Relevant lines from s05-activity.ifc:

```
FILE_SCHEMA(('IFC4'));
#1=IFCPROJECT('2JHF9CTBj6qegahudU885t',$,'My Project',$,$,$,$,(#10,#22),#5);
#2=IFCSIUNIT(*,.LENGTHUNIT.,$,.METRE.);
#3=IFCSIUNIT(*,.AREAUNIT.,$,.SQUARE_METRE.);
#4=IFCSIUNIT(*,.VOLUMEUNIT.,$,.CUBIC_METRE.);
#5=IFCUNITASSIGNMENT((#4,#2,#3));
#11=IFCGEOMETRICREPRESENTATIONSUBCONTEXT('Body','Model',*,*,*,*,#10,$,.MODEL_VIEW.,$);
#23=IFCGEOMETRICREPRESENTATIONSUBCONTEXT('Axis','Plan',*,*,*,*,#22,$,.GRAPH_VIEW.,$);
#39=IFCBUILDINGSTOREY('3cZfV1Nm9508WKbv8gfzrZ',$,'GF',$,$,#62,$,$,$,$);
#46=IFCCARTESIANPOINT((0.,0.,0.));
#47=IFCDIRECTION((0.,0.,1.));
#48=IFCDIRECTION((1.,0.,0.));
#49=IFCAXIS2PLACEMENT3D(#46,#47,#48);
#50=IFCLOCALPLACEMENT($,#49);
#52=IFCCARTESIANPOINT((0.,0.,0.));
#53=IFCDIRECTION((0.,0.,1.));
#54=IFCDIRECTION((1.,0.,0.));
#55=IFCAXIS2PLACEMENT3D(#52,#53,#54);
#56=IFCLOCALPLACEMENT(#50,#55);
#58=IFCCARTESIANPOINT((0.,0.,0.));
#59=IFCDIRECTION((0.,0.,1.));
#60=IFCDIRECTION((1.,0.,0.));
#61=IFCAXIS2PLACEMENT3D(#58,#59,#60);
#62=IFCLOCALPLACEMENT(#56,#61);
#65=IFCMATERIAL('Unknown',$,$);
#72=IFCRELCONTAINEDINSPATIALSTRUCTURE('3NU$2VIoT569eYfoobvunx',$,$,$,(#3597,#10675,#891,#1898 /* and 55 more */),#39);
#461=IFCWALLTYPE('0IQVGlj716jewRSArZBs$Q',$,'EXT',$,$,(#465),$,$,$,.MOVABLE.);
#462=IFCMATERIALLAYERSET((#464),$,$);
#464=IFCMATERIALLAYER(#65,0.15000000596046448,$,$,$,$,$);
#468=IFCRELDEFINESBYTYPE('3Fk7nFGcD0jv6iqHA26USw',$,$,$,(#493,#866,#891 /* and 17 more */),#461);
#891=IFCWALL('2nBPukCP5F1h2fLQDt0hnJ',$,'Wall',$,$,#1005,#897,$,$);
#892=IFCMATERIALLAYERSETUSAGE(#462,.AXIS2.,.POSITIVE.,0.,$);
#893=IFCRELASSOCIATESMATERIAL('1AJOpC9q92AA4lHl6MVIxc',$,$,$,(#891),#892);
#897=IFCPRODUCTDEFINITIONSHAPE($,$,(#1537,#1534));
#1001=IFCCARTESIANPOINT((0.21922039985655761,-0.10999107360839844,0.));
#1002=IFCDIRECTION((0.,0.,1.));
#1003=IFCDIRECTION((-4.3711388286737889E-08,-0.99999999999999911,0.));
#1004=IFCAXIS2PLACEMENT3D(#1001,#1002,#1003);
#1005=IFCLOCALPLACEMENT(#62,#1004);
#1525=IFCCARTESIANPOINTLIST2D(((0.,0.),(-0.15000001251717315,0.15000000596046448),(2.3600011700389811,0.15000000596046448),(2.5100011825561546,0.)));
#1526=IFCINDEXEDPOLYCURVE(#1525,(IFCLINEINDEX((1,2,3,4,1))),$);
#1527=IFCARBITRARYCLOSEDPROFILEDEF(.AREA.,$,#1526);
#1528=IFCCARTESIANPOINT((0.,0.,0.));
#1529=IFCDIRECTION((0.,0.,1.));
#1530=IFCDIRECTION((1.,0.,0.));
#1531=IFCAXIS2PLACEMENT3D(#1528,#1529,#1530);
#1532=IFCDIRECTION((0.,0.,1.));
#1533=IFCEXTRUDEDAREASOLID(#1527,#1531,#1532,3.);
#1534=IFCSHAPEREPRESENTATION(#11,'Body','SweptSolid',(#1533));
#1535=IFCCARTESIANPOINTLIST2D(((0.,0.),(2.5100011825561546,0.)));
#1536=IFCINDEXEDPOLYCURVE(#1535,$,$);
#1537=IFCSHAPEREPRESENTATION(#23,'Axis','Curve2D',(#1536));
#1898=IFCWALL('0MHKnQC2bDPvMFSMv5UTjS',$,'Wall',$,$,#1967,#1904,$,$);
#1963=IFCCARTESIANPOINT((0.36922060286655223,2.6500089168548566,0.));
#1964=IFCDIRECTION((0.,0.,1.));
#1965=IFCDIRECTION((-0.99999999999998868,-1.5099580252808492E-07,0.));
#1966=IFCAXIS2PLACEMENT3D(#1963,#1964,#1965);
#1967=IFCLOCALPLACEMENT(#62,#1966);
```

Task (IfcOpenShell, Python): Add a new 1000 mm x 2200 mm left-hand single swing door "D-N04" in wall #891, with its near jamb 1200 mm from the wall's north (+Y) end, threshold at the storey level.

```python
import numpy as np
import ifcopenshell
import ifcopenshell.api.feature
import ifcopenshell.api.geometry
import ifcopenshell.api.root
import ifcopenshell.api.spatial
import ifcopenshell.geom
import ifcopenshell.util.element
import ifcopenshell.util.placement
import ifcopenshell.util.representation
import ifcopenshell.util.shape
import ifcopenshell.util.unit

model = ifcopenshell.open("s05-activity.ifc")
unit_scale = ifcopenshell.util.unit.calculate_unit_scale(model)
settings = ifcopenshell.geom.settings()


def volume(element):
    """Net volume in cubic metres, openings subtracted."""
    shape = ifcopenshell.geom.create_shape(settings, element)
    return ifcopenshell.util.shape.get_volume(shape.geometry)


wall = model.by_guid("2nBPukCP5F1h2fLQDt0hnJ")
storey = ifcopenshell.util.element.get_container(wall, ifc_class="IfcBuildingStorey")
context = ifcopenshell.util.representation.get_context(model, "Model", "Body", "MODEL_VIEW")
before = volume(wall)

width, height, from_end, sill = 1, 2.2, 1.2, 0.0  # metres

# The wall runs along its own X axis, and the end named is its -X end.
wall_shape = ifcopenshell.geom.create_shape(settings, wall)
x, y, z = ifcopenshell.util.shape.get_vertices(wall_shape.geometry).T
start = x.min() + from_end
face, thickness = float(y.min()), float(y.max() - y.min())
wall_matrix = ifcopenshell.util.placement.get_local_placement(wall.ObjectPlacement)
level = ifcopenshell.util.placement.get_local_placement(storey.ObjectPlacement)[2, 3]


def in_wall(x, y):
    """Placement at x, y metres in the wall's axes, at sill height."""
    matrix = wall_matrix.copy()
    matrix[:, 3] = wall_matrix @ np.array([x / unit_scale, y / unit_scale, 0.0, 1.0])
    matrix[2, 3] = level + sill / unit_scale
    return matrix


# Opening: a box that overshoots both wall faces by 50 mm.
opening = ifcopenshell.api.root.create_entity(model, ifc_class="IfcOpeningElement", predefined_type="OPENING")
box = ifcopenshell.api.geometry.add_wall_representation(
    model, context=context, length=width, height=height, thickness=thickness + 0.1
)
ifcopenshell.api.geometry.assign_representation(model, product=opening, representation=box)
ifcopenshell.api.geometry.edit_object_placement(model, product=opening, matrix=in_wall(start, face - 0.05), is_si=False)
ifcopenshell.api.feature.add_feature(model, feature=opening, element=wall)

door = ifcopenshell.api.root.create_entity(model, ifc_class="IfcDoor", name="D-N04", predefined_type="DOOR")
door.OverallWidth, door.OverallHeight = width / unit_scale, height / unit_scale
door.OperationType = "SINGLE_SWING_LEFT"
body = ifcopenshell.api.geometry.add_door_representation(
    model,
    context=context,
    overall_width=door.OverallWidth,
    overall_height=door.OverallHeight,
    operation_type="SINGLE_SWING_LEFT",
    lining_properties={"LiningDepth": thickness / unit_scale, "ThresholdDepth": thickness / unit_scale},
)
ifcopenshell.api.geometry.assign_representation(model, product=door, representation=body)
ifcopenshell.api.spatial.assign_container(model, products=[door], relating_structure=storey)
ifcopenshell.api.feature.add_filling(model, opening=opening, element=door)

# The lining spans the wall, so the door starts at the wall face.
ifcopenshell.api.geometry.edit_object_placement(model, product=door, matrix=in_wall(start, face), is_si=False)

after = volume(wall)

print(f"wall volume {before:.3f} -> {after:.3f} m3")

model.write("s05-activity_updated.ifc")
```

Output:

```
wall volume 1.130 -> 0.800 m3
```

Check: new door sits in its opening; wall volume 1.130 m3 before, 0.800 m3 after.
